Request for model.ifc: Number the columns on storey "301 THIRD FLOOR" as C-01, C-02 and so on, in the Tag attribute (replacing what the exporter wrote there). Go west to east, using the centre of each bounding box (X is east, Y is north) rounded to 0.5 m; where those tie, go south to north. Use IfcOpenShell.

First a look at what the model holds.

```python
import ifcopenshell
import ifcopenshell.util.element
import ifcopenshell.util.placement

model = ifcopenshell.open("model.ifc")
print(model.schema)
storey = next(s for s in model.by_type("IfcBuildingStorey") if s.Name == "301 THIRD FLOOR")
columns = [e for e in ifcopenshell.util.element.get_decomposition(storey) if e.is_a("IfcColumn")]
for e in sorted(columns, key=lambda e: e.id()):
    origin = ifcopenshell.util.placement.get_local_placement(e.ObjectPlacement)[:3, 3]
    print(e.id(), e.Tag, e.Name, origin.round(2) + 0.0, sep=" | ")
```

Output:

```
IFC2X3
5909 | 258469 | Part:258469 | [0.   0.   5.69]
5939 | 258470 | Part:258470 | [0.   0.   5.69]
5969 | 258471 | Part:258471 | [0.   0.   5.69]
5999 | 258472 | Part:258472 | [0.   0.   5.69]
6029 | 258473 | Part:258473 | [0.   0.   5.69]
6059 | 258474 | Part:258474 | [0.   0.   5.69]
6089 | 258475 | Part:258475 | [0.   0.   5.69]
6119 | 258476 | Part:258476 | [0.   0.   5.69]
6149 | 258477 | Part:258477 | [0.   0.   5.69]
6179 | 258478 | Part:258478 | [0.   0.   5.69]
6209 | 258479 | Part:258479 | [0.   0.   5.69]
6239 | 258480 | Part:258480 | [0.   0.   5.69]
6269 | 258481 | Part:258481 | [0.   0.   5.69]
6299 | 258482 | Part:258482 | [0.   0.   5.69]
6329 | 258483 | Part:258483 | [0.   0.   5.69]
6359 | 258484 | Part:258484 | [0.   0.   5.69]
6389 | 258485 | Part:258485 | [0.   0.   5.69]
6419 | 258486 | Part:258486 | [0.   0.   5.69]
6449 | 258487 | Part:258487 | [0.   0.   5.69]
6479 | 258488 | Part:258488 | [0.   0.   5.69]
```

```python
import ifcopenshell
import ifcopenshell.geom
import ifcopenshell.util.element
import ifcopenshell.util.shape

model = ifcopenshell.open("model.ifc")
settings = ifcopenshell.geom.settings()
settings.set("use-world-coords", True)


def centre(element):
    shape = ifcopenshell.geom.create_shape(settings, element)
    return ifcopenshell.util.shape.get_bbox_centroid(shape.geometry)


storey = next(s for s in model.by_type("IfcBuildingStorey") if s.Name == "301 THIRD FLOOR")
columns = [e for e in ifcopenshell.util.element.get_decomposition(storey) if e.is_a("IfcColumn")]

# Insertion points can sit at a corner or the storey origin, so sort by the geometry (in metres).
centres = {e: centre(e) for e in columns}
columns.sort(key=lambda e: (round(centres[e][0] / 0.5), centres[e][1]))

for i, e in enumerate(columns, start=1):
    number = f"C-{i:02d}"
    e.Tag = number
    print(e.id(), number)

model.write("model_rev.ifc")
```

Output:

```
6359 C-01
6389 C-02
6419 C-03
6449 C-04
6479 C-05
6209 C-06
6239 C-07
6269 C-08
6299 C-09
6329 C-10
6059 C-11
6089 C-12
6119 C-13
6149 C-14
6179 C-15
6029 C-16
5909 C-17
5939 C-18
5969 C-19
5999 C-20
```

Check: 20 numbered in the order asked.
